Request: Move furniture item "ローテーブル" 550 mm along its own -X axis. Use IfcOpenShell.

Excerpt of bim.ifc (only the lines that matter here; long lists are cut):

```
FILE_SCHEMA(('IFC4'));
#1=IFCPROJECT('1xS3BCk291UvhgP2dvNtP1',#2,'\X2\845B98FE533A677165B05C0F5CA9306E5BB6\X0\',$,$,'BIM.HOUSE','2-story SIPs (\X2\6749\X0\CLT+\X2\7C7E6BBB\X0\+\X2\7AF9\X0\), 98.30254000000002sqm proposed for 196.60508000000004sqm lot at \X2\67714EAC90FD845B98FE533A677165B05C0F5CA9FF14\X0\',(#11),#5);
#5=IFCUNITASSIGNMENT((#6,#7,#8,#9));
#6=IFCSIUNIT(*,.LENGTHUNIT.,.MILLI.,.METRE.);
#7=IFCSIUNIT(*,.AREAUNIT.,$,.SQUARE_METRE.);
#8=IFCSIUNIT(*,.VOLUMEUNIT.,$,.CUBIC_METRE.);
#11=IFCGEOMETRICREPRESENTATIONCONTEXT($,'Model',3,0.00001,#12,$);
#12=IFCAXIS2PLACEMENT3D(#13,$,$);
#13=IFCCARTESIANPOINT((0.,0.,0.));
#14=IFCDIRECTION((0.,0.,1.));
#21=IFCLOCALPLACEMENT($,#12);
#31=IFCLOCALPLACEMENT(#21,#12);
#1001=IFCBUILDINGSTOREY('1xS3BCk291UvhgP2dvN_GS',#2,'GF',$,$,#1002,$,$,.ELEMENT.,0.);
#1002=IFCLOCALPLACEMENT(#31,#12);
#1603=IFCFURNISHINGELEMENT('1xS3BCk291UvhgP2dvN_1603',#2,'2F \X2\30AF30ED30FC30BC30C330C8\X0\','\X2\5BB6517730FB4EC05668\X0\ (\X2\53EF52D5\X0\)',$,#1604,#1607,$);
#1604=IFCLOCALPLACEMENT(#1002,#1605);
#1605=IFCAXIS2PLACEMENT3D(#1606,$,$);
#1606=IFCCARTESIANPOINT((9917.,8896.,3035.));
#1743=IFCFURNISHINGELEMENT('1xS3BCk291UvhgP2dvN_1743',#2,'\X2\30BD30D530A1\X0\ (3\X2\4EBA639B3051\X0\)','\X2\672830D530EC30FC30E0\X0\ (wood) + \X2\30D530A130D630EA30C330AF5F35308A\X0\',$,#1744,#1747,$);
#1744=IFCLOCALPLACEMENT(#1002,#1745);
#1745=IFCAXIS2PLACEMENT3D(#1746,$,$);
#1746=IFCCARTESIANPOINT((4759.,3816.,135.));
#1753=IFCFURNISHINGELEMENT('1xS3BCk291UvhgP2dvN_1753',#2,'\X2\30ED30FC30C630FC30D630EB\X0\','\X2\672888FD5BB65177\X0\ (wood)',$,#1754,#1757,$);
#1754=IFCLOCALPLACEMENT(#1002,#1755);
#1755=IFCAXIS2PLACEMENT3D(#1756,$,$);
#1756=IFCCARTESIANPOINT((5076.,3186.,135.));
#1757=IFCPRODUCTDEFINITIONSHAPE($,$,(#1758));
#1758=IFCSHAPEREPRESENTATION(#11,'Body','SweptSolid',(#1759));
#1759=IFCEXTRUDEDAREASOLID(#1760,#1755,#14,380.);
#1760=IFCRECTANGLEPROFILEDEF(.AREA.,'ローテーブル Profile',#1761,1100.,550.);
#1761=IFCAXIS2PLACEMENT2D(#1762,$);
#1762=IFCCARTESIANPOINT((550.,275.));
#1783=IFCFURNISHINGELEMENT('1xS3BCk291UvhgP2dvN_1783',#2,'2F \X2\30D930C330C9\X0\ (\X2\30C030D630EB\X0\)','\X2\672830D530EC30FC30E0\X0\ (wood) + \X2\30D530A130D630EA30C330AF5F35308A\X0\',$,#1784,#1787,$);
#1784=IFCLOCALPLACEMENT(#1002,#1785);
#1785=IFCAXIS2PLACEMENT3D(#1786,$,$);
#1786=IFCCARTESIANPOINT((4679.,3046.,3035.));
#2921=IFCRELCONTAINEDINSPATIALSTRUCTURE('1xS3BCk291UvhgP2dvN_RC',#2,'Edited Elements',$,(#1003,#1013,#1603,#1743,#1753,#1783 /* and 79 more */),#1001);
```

```python
import ifcopenshell
import ifcopenshell.api.geometry
import ifcopenshell.util.placement

model = ifcopenshell.open("bim.ifc")

item = model.by_id(1753)
matrix = ifcopenshell.util.placement.get_local_placement(item.ObjectPlacement)
matrix[:3, 3] -= matrix[:3, 0] * 550.0
ifcopenshell.api.geometry.edit_object_placement(model, product=item, matrix=matrix, is_si=False)

print(ifcopenshell.util.placement.get_local_placement(item.ObjectPlacement).round(3) + 0.0)

model.write("bim_v2.ifc")
```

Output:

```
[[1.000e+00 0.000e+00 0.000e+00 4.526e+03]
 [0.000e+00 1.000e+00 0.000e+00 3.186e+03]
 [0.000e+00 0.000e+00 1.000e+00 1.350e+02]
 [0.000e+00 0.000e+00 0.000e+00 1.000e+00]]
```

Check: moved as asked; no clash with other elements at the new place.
